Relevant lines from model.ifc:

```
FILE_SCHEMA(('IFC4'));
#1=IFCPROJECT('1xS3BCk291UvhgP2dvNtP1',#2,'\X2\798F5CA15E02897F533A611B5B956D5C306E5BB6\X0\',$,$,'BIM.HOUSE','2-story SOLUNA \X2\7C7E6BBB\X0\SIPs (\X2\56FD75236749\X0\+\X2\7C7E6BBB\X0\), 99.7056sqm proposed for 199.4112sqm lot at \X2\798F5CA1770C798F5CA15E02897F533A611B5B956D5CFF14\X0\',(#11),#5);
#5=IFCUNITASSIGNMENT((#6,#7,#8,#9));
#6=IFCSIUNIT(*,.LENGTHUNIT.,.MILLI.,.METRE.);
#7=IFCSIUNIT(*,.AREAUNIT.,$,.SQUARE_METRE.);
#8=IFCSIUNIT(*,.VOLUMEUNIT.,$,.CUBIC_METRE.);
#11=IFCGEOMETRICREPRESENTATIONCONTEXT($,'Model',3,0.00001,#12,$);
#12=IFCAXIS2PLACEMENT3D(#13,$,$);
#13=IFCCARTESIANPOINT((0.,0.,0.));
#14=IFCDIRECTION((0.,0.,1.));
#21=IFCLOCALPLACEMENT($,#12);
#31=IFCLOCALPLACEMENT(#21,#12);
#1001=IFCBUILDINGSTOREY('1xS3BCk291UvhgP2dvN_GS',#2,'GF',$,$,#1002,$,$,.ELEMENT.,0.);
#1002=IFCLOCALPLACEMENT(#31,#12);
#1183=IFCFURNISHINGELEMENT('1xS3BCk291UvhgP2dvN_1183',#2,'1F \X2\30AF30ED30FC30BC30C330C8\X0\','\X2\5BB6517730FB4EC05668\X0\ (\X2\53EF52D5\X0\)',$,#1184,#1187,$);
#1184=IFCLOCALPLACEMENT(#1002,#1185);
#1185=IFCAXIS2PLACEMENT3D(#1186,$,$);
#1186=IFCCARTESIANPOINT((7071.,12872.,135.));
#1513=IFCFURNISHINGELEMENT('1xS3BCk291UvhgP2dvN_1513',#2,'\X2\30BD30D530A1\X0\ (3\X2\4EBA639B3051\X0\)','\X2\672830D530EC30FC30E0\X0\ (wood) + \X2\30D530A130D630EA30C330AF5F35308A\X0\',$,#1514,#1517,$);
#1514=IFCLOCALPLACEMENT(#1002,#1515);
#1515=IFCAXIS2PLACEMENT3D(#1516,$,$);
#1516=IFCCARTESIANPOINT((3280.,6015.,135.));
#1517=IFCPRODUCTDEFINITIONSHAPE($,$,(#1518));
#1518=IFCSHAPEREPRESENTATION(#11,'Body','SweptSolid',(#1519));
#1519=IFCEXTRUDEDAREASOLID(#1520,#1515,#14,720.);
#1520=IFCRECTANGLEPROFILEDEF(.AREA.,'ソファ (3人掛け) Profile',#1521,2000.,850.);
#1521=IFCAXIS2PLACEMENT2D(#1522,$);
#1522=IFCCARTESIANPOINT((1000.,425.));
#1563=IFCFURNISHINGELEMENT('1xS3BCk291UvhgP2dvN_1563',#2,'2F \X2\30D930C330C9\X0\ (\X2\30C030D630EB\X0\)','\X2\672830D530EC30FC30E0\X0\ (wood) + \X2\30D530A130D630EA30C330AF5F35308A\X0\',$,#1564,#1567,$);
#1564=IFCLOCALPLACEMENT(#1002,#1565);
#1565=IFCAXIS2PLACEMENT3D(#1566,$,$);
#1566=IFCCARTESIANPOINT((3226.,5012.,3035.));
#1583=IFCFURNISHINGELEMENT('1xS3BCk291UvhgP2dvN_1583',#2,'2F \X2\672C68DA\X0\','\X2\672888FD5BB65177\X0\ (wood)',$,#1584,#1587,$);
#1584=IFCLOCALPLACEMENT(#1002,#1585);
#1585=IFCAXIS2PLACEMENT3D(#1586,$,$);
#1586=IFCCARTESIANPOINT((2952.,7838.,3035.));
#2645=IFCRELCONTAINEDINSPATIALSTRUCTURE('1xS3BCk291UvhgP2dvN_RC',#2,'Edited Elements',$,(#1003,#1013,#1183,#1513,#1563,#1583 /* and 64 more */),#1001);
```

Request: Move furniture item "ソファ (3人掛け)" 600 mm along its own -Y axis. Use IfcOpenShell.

```python
import ifcopenshell
import ifcopenshell.api.geometry
import ifcopenshell.util.placement

model = ifcopenshell.open("model.ifc")

item = model.by_guid("1xS3BCk291UvhgP2dvN_1513")
matrix = ifcopenshell.util.placement.get_local_placement(item.ObjectPlacement)
matrix[:3, 3] -= matrix[:3, 1] * 600.0
ifcopenshell.api.geometry.edit_object_placement(model, product=item, matrix=matrix, is_si=False)

print(ifcopenshell.util.placement.get_local_placement(item.ObjectPlacement).round(3) + 0.0)

model.write("model_rev.ifc")
```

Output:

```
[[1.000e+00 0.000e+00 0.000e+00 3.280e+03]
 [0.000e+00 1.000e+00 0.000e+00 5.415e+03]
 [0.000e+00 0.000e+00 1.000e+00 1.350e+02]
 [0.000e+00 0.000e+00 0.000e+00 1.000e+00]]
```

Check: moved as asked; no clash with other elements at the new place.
